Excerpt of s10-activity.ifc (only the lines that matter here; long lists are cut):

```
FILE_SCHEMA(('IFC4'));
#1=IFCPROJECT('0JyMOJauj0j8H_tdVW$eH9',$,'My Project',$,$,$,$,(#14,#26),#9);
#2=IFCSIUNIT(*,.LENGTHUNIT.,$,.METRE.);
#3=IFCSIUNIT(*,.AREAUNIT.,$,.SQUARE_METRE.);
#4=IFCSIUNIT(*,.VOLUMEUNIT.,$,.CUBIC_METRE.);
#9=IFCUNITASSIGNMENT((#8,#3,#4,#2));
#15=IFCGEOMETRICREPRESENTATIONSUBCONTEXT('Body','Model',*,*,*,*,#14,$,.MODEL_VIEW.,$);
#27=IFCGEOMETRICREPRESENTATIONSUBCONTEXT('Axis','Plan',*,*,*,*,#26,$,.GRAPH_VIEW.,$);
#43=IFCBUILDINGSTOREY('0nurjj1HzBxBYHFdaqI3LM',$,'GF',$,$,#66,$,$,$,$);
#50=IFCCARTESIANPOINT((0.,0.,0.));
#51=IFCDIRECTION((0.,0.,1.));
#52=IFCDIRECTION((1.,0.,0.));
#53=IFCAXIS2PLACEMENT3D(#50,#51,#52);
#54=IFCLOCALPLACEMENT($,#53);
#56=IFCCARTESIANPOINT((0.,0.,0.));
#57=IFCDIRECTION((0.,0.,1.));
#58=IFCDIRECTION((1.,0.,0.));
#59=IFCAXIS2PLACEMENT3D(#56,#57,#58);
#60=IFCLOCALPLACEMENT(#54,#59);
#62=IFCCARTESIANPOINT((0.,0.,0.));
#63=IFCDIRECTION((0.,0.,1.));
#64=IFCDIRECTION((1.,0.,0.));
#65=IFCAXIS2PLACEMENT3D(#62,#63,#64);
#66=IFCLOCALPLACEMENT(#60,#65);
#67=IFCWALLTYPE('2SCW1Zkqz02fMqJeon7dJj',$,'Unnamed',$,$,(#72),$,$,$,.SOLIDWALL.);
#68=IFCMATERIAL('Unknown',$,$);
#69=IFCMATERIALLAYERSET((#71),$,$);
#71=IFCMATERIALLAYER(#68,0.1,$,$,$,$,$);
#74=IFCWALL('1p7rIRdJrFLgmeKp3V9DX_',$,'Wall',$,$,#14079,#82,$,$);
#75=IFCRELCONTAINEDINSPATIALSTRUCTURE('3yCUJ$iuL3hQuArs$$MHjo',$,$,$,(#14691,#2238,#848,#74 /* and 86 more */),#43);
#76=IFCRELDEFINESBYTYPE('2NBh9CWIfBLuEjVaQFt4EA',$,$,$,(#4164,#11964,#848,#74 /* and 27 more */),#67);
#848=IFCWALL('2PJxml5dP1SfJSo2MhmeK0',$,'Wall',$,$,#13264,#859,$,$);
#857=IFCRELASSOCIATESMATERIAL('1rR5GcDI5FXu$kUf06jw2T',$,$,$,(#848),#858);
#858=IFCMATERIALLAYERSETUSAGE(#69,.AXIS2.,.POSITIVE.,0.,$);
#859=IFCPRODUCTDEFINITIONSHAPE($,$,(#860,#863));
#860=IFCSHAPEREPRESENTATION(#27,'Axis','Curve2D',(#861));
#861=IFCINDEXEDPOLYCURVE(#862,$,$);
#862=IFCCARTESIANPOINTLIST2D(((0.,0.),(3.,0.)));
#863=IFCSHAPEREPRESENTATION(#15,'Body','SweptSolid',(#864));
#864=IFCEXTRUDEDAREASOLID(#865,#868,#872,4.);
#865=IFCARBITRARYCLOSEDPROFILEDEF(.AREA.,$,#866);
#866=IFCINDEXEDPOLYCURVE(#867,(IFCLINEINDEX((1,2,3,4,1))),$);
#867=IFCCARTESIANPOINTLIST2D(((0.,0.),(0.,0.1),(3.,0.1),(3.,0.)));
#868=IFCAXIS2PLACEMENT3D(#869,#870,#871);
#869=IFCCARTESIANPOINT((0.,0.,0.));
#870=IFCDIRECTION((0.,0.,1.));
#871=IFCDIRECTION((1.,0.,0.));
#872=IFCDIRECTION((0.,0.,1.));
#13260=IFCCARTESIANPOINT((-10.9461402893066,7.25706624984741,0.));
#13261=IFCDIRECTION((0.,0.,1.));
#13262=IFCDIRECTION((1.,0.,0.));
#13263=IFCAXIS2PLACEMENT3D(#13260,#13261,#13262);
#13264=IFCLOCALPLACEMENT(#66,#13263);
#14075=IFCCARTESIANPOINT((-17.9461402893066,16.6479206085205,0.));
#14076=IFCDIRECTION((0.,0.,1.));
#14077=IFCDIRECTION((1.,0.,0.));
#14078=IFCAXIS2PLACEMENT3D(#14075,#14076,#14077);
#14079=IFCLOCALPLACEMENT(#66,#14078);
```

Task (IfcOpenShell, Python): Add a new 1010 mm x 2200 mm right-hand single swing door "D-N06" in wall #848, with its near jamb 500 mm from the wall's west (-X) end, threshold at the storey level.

```python
import numpy as np
import ifcopenshell
import ifcopenshell.api.feature
import ifcopenshell.api.geometry
import ifcopenshell.api.root
import ifcopenshell.api.spatial
import ifcopenshell.geom
import ifcopenshell.util.element
import ifcopenshell.util.placement
import ifcopenshell.util.representation
import ifcopenshell.util.shape
import ifcopenshell.util.unit

model = ifcopenshell.open("s10-activity.ifc")
unit_scale = ifcopenshell.util.unit.calculate_unit_scale(model)
settings = ifcopenshell.geom.settings()


def volume(element):
    """Net volume in cubic metres, openings subtracted."""
    shape = ifcopenshell.geom.create_shape(settings, element)
    return ifcopenshell.util.shape.get_volume(shape.geometry)


wall = model.by_guid("2PJxml5dP1SfJSo2MhmeK0")
storey = ifcopenshell.util.element.get_container(wall, ifc_class="IfcBuildingStorey")
context = ifcopenshell.util.representation.get_context(model, "Model", "Body", "MODEL_VIEW")
before = volume(wall)

width, height, from_end, sill = 1.01, 2.2, 0.5, 0.0  # metres

# The wall runs along its own X axis, and the end named is its -X end.
wall_shape = ifcopenshell.geom.create_shape(settings, wall)
x, y, z = ifcopenshell.util.shape.get_vertices(wall_shape.geometry).T
start = x.min() + from_end
face, thickness = float(y.min()), float(y.max() - y.min())
wall_matrix = ifcopenshell.util.placement.get_local_placement(wall.ObjectPlacement)
level = ifcopenshell.util.placement.get_local_placement(storey.ObjectPlacement)[2, 3]


def in_wall(x, y):
    """Placement at x, y metres in the wall's axes, at sill height."""
    matrix = wall_matrix.copy()
    matrix[:, 3] = wall_matrix @ np.array([x / unit_scale, y / unit_scale, 0.0, 1.0])
    matrix[2, 3] = level + sill / unit_scale
    return matrix


# Opening: a box that overshoots both wall faces by 50 mm.
opening = ifcopenshell.api.root.create_entity(model, ifc_class="IfcOpeningElement", predefined_type="OPENING")
box = ifcopenshell.api.geometry.add_wall_representation(
    model, context=context, length=width, height=height, thickness=thickness + 0.1
)
ifcopenshell.api.geometry.assign_representation(model, product=opening, representation=box)
ifcopenshell.api.geometry.edit_object_placement(model, product=opening, matrix=in_wall(start, face - 0.05), is_si=False)
ifcopenshell.api.feature.add_feature(model, feature=opening, element=wall)

door = ifcopenshell.api.root.create_entity(model, ifc_class="IfcDoor", name="D-N06", predefined_type="DOOR")
door.OverallWidth, door.OverallHeight = width / unit_scale, height / unit_scale
door.OperationType = "SINGLE_SWING_RIGHT"
body = ifcopenshell.api.geometry.add_door_representation(
    model,
    context=context,
    overall_width=door.OverallWidth,
    overall_height=door.OverallHeight,
    operation_type="SINGLE_SWING_RIGHT",
    lining_properties={"LiningDepth": thickness / unit_scale, "ThresholdDepth": thickness / unit_scale},
)
ifcopenshell.api.geometry.assign_representation(model, product=door, representation=body)
ifcopenshell.api.spatial.assign_container(model, products=[door], relating_structure=storey)
ifcopenshell.api.feature.add_filling(model, opening=opening, element=door)

# The lining spans the wall, so the door starts at the wall face.
ifcopenshell.api.geometry.edit_object_placement(model, product=door, matrix=in_wall(start, face), is_si=False)

after = volume(wall)

print(f"wall volume {before:.3f} -> {after:.3f} m3")

model.write("s10-activity_rev.ifc")
```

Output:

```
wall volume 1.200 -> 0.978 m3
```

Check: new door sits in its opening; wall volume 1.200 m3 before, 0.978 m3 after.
